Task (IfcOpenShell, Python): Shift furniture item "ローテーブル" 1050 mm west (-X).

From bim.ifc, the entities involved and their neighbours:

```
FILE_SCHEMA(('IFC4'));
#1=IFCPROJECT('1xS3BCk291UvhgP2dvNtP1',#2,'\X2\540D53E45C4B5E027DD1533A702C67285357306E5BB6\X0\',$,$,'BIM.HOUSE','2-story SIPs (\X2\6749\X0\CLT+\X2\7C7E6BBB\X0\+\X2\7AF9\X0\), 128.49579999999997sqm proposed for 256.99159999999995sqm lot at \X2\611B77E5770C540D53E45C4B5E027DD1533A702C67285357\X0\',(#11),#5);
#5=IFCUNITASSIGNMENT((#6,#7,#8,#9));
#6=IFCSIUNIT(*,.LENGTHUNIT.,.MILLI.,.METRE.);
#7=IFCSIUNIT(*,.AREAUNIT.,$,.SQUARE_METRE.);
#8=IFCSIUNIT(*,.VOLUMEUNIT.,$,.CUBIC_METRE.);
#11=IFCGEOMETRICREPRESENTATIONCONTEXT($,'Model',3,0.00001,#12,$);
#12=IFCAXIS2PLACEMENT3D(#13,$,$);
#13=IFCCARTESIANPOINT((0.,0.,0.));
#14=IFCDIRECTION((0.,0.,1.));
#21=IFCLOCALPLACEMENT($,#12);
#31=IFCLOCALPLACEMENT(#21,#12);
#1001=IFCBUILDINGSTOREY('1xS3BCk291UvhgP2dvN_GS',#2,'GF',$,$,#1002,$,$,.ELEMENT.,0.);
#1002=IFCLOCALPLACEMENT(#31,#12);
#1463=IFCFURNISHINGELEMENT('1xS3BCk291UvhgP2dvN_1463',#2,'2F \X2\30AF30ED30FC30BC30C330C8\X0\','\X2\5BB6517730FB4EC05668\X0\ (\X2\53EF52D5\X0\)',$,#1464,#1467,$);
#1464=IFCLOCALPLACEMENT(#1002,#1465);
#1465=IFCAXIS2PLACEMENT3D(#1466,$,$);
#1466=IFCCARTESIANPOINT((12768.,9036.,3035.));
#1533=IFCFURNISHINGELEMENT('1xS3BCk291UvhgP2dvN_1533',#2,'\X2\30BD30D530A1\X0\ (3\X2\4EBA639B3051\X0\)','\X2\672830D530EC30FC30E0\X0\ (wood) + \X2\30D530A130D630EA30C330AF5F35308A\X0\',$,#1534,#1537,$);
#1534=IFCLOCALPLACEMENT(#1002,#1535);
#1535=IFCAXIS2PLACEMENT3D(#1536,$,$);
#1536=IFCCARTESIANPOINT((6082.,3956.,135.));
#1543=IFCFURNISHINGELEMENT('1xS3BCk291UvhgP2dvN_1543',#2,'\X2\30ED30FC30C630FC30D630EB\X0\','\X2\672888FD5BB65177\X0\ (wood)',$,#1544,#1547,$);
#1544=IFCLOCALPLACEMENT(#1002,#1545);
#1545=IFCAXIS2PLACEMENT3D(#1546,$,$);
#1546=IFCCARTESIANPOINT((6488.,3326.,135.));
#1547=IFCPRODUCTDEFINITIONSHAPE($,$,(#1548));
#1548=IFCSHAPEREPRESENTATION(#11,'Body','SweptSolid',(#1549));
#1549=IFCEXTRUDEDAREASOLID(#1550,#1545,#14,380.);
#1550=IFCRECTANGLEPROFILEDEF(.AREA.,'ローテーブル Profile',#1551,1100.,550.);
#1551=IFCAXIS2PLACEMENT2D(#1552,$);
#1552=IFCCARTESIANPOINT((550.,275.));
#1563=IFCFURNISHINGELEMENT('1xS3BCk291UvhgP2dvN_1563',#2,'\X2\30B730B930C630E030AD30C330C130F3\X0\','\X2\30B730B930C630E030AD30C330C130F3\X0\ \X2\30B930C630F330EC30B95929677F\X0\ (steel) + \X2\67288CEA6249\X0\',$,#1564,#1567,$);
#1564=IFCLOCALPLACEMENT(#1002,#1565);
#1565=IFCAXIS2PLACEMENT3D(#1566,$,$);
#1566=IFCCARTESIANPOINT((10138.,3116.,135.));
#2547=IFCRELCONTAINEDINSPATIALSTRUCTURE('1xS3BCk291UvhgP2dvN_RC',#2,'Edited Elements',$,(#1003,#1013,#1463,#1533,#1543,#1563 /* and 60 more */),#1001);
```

```python
import ifcopenshell
import ifcopenshell.api.geometry
import ifcopenshell.util.placement
import ifcopenshell.util.unit

model = ifcopenshell.open("bim.ifc")
unit_scale = ifcopenshell.util.unit.calculate_unit_scale(model)

item = model.by_guid("1xS3BCk291UvhgP2dvN_1543")
matrix = ifcopenshell.util.placement.get_local_placement(item.ObjectPlacement)
matrix[0, 3] -= 1.05 / unit_scale
ifcopenshell.api.geometry.edit_object_placement(model, product=item, matrix=matrix, is_si=False)

print(ifcopenshell.util.placement.get_local_placement(item.ObjectPlacement).round(3) + 0.0)

model.write("bim_edited.ifc")
```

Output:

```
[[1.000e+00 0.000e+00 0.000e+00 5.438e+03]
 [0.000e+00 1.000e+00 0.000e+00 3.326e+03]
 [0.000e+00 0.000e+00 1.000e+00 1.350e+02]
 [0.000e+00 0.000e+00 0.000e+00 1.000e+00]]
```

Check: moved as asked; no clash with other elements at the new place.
